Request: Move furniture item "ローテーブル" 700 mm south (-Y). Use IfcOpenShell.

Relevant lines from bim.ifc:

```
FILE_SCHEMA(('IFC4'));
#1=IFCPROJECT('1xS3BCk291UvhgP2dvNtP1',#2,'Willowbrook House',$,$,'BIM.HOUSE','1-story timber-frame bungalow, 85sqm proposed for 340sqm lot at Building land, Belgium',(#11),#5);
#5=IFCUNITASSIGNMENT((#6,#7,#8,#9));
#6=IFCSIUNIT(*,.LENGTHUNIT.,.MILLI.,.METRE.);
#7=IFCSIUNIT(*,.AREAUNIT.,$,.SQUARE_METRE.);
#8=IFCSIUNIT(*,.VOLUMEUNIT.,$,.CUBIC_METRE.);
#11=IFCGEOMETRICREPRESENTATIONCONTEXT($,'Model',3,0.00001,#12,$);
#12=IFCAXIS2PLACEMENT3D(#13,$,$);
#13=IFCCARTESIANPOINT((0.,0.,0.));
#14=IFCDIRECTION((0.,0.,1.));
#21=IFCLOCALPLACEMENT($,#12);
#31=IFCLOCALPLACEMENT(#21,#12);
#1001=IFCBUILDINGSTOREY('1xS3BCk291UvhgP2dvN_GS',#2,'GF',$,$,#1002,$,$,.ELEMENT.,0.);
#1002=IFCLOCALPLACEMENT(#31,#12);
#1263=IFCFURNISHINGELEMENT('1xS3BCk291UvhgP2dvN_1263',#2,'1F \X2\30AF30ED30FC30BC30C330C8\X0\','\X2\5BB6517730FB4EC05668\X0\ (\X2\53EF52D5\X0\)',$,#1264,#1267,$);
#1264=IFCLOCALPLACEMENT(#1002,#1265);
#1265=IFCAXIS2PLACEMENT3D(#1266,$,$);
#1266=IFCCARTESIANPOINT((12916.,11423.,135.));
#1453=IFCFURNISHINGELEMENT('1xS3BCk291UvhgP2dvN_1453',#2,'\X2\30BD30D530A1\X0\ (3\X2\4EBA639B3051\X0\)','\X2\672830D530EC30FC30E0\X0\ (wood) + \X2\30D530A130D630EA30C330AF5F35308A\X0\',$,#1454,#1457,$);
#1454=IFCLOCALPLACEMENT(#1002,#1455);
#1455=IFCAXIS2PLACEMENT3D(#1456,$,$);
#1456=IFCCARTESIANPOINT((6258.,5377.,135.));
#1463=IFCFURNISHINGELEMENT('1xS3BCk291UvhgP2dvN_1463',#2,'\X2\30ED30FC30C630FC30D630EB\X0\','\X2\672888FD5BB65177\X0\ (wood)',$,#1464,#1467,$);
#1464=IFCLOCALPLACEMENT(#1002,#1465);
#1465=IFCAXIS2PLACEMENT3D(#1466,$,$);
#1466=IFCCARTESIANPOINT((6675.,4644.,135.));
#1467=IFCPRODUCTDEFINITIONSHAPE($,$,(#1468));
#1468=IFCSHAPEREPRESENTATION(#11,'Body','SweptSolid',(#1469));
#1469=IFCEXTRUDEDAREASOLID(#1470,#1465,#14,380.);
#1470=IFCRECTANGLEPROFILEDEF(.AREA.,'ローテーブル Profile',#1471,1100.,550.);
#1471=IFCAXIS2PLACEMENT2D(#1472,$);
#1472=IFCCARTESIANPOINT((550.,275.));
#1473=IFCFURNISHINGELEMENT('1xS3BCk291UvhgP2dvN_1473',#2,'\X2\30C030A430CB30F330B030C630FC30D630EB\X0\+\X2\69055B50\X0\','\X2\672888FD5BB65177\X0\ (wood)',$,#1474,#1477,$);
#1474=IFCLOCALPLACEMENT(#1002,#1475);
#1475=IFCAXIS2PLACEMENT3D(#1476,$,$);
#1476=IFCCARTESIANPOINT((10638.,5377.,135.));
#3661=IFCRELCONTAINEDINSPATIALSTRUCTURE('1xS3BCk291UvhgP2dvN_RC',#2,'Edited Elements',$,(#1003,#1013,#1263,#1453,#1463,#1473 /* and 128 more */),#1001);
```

```python
import ifcopenshell
import ifcopenshell.api.geometry
import ifcopenshell.util.placement

model = ifcopenshell.open("bim.ifc")

item = model.by_id(1463)
matrix = ifcopenshell.util.placement.get_local_placement(item.ObjectPlacement)
matrix[1, 3] -= 700.0
ifcopenshell.api.geometry.edit_object_placement(model, product=item, matrix=matrix, is_si=False)

print(ifcopenshell.util.placement.get_local_placement(item.ObjectPlacement).round(3) + 0.0)

model.write("bim_v2.ifc")
```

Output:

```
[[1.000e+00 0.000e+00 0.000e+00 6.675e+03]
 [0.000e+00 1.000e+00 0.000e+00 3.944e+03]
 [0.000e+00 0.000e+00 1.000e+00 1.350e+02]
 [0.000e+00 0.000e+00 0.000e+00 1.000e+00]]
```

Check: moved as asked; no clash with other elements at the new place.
